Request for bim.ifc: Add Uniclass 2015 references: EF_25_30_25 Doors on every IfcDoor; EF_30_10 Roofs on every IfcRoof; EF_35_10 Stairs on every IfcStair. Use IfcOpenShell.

First a look at what the model holds.

```python
import ifcopenshell

model = ifcopenshell.open("bim.ifc")
print(model.schema)
print("classifications:", [c.Name for c in model.by_type("IfcClassification")])
for ifc_class in ("IfcDoor", "IfcRoof", "IfcStair", "IfcWall", "IfcWindow"):
    print(ifc_class, len(model.by_type(ifc_class)))
```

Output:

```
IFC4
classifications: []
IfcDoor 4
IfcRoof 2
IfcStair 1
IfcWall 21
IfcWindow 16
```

```python
import ifcopenshell
import ifcopenshell.api.classification

model = ifcopenshell.open("bim.ifc")

system = ifcopenshell.api.classification.add_classification(model, classification="Uniclass 2015")

codes = {
    "IfcDoor": ("EF_25_30_25", "Doors"),
    "IfcRoof": ("EF_30_10", "Roofs"),
    "IfcStair": ("EF_35_10", "Stairs"),
}
for ifc_class, (code, name) in codes.items():
    products = model.by_type(ifc_class)
    ifcopenshell.api.classification.add_reference(
        model, products=products, classification=system, identification=code, name=name
    )
    print(code, len(products))

model.write("bim-out.ifc")
```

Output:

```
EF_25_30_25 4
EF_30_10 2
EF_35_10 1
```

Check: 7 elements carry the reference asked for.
